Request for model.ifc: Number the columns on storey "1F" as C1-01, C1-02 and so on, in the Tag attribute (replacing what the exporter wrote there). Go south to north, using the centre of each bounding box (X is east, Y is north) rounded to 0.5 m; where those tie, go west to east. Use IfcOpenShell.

First a look at what the model holds.

```python
import ifcopenshell
import ifcopenshell.util.element
import ifcopenshell.util.placement

model = ifcopenshell.open("model.ifc")
print(model.schema)
storey = next(s for s in model.by_type("IfcBuildingStorey") if s.Name == "1F")
columns = [e for e in ifcopenshell.util.element.get_decomposition(storey) if e.is_a("IfcColumn")]
for e in sorted(columns, key=lambda e: e.id()):
    origin = ifcopenshell.util.placement.get_local_placement(e.ObjectPlacement)[:3, 3]
    print(e.id(), e.Tag, e.Name, origin.round(2) + 0.0, sep=" | ")
```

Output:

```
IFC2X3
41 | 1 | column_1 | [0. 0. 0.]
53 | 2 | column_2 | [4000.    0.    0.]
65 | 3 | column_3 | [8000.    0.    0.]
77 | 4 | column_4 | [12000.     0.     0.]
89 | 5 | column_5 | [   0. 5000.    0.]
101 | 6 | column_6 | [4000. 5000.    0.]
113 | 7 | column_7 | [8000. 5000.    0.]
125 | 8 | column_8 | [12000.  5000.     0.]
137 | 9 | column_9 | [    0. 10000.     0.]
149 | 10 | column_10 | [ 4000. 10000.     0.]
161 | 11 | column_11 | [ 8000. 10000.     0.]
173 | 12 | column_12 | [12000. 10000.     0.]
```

```python
import ifcopenshell
import ifcopenshell.geom
import ifcopenshell.util.element
import ifcopenshell.util.shape

model = ifcopenshell.open("model.ifc")
settings = ifcopenshell.geom.settings()
settings.set("use-world-coords", True)


def centre(element):
    shape = ifcopenshell.geom.create_shape(settings, element)
    return ifcopenshell.util.shape.get_bbox_centroid(shape.geometry)


storey = next(s for s in model.by_type("IfcBuildingStorey") if s.Name == "1F")
columns = [e for e in ifcopenshell.util.element.get_decomposition(storey) if e.is_a("IfcColumn")]

# Insertion points can sit at a corner or the storey origin, so sort by the geometry (in metres).
centres = {e: centre(e) for e in columns}
columns.sort(key=lambda e: (round(centres[e][1] / 0.5), centres[e][0]))

for i, e in enumerate(columns, start=1):
    number = f"C1-{i:02d}"
    e.Tag = number
    print(e.id(), number)

model.write("model-out.ifc")
```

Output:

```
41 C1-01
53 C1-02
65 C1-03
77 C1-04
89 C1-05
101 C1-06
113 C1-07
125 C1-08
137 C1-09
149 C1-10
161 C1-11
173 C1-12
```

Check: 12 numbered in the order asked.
